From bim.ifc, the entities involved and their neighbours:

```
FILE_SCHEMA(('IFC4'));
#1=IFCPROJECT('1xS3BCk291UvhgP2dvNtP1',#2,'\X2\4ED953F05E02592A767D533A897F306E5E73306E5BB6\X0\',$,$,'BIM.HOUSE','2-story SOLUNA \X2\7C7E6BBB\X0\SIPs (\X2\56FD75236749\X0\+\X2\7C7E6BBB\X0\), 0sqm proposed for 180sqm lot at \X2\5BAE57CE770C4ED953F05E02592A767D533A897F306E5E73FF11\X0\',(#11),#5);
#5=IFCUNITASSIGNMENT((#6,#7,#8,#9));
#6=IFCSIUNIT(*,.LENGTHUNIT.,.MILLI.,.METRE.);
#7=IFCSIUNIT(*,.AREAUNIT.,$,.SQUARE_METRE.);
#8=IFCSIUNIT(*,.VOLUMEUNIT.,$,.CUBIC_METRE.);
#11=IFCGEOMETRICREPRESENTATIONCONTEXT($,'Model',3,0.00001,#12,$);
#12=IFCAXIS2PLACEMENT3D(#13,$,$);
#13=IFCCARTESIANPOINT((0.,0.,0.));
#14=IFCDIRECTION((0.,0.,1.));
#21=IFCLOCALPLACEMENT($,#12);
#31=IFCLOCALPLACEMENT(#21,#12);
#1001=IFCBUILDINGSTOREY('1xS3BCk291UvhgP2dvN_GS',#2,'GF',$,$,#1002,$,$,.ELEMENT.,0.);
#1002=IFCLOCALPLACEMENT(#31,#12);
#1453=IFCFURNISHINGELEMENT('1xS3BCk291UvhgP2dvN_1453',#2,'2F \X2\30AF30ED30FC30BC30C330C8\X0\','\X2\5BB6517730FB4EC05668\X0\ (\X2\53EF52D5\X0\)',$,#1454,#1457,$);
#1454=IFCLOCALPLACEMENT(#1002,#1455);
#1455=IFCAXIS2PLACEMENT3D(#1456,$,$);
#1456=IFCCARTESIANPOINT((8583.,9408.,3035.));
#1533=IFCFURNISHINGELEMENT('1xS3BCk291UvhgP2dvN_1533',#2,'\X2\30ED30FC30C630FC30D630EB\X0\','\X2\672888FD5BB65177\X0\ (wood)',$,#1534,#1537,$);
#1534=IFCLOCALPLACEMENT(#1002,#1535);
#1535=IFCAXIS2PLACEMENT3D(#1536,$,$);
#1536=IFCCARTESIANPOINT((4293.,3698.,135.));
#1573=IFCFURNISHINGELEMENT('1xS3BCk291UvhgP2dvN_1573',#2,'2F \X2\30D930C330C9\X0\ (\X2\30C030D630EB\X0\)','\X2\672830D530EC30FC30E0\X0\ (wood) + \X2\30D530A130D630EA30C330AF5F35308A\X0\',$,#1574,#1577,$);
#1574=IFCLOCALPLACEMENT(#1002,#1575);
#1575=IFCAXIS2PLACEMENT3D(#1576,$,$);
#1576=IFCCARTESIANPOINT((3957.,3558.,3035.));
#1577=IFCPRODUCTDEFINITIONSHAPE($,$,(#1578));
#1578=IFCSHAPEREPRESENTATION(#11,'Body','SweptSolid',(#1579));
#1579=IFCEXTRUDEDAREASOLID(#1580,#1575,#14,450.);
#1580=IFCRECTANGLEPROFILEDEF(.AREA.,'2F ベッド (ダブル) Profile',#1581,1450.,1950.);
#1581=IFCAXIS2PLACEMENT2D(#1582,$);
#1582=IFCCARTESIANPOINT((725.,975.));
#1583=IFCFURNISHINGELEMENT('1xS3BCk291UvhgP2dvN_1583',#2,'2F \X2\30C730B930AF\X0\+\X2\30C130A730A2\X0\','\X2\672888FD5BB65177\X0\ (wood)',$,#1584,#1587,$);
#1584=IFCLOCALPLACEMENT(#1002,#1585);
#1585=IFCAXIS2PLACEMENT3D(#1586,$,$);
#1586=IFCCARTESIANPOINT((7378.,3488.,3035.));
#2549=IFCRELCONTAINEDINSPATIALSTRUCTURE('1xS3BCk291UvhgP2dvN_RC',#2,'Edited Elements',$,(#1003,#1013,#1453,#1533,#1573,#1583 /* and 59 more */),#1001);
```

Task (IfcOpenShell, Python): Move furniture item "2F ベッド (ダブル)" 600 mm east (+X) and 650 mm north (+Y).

```python
import ifcopenshell
import ifcopenshell.api.geometry
import ifcopenshell.util.placement
import ifcopenshell.util.unit

model = ifcopenshell.open("bim.ifc")
unit_scale = ifcopenshell.util.unit.calculate_unit_scale(model)

item = model.by_id(1573)
matrix = ifcopenshell.util.placement.get_local_placement(item.ObjectPlacement)
matrix[0, 3] += 0.6 / unit_scale
matrix[1, 3] += 0.65 / unit_scale
ifcopenshell.api.geometry.edit_object_placement(model, product=item, matrix=matrix, is_si=False)

print(ifcopenshell.util.placement.get_local_placement(item.ObjectPlacement).round(3) + 0.0)

model.write("bim_updated.ifc")
```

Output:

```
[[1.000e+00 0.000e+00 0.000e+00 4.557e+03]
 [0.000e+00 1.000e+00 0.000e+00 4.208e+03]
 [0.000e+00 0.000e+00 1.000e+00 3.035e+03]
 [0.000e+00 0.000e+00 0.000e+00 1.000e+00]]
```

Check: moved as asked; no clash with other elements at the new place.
